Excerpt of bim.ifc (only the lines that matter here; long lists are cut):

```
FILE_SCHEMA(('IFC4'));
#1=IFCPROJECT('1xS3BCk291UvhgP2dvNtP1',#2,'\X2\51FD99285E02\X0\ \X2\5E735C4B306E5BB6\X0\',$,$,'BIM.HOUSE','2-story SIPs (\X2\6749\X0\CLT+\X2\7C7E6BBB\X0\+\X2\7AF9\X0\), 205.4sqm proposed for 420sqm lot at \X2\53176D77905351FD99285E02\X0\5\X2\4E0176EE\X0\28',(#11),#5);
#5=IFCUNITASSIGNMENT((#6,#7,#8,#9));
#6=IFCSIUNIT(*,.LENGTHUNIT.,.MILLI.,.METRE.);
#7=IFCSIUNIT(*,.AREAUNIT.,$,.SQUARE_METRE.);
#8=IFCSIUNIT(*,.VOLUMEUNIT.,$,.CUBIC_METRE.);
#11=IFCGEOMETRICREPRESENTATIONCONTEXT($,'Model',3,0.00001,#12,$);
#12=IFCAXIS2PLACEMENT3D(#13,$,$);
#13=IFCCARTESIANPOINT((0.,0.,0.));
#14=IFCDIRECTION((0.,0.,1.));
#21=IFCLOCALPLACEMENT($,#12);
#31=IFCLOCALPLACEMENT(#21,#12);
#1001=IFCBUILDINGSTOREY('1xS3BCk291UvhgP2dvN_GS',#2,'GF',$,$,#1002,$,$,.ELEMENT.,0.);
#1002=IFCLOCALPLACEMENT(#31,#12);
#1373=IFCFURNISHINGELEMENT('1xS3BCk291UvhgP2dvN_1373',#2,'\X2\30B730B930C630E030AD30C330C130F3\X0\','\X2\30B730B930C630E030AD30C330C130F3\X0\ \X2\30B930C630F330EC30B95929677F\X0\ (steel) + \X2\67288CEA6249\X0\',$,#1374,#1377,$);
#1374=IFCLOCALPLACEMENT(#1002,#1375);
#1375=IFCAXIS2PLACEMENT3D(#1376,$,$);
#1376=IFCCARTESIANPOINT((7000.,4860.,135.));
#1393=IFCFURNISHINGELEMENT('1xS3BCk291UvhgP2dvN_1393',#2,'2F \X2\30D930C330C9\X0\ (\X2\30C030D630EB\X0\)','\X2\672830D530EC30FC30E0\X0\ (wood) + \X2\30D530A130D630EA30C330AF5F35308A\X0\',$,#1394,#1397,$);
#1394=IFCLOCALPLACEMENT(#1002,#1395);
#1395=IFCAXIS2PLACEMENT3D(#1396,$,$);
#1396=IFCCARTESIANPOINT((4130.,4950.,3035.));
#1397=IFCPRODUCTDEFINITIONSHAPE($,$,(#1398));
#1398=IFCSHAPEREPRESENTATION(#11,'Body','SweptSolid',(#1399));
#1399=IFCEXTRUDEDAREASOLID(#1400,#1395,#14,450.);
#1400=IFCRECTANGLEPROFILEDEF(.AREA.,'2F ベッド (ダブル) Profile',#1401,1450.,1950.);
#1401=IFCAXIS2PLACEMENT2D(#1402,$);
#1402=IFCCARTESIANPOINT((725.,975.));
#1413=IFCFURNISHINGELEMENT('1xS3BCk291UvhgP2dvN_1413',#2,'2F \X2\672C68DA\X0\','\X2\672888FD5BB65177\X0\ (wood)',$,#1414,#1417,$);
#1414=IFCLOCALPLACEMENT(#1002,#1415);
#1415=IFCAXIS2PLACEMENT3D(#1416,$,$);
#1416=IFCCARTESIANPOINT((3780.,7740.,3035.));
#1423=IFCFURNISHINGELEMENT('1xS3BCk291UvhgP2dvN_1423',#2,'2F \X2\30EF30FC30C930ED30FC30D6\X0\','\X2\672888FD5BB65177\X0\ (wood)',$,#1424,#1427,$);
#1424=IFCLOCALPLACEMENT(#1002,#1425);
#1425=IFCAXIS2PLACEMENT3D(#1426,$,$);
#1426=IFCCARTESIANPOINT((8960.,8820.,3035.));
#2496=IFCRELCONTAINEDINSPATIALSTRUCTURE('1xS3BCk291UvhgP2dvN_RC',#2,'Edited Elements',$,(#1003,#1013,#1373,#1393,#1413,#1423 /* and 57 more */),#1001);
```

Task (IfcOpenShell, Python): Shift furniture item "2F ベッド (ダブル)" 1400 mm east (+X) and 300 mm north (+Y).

```python
import ifcopenshell
import ifcopenshell.api.geometry
import ifcopenshell.util.placement

model = ifcopenshell.open("bim.ifc")

item = model.by_guid("1xS3BCk291UvhgP2dvN_1393")
matrix = ifcopenshell.util.placement.get_local_placement(item.ObjectPlacement)
matrix[0, 3] += 1400.0
matrix[1, 3] += 300.0
ifcopenshell.api.geometry.edit_object_placement(model, product=item, matrix=matrix, is_si=False)

print(ifcopenshell.util.placement.get_local_placement(item.ObjectPlacement).round(3) + 0.0)

model.write("bim_v2.ifc")
```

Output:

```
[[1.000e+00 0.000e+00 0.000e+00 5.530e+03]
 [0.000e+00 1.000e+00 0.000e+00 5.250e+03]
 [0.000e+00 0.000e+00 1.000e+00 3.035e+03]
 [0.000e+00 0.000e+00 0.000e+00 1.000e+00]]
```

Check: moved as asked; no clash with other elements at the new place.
